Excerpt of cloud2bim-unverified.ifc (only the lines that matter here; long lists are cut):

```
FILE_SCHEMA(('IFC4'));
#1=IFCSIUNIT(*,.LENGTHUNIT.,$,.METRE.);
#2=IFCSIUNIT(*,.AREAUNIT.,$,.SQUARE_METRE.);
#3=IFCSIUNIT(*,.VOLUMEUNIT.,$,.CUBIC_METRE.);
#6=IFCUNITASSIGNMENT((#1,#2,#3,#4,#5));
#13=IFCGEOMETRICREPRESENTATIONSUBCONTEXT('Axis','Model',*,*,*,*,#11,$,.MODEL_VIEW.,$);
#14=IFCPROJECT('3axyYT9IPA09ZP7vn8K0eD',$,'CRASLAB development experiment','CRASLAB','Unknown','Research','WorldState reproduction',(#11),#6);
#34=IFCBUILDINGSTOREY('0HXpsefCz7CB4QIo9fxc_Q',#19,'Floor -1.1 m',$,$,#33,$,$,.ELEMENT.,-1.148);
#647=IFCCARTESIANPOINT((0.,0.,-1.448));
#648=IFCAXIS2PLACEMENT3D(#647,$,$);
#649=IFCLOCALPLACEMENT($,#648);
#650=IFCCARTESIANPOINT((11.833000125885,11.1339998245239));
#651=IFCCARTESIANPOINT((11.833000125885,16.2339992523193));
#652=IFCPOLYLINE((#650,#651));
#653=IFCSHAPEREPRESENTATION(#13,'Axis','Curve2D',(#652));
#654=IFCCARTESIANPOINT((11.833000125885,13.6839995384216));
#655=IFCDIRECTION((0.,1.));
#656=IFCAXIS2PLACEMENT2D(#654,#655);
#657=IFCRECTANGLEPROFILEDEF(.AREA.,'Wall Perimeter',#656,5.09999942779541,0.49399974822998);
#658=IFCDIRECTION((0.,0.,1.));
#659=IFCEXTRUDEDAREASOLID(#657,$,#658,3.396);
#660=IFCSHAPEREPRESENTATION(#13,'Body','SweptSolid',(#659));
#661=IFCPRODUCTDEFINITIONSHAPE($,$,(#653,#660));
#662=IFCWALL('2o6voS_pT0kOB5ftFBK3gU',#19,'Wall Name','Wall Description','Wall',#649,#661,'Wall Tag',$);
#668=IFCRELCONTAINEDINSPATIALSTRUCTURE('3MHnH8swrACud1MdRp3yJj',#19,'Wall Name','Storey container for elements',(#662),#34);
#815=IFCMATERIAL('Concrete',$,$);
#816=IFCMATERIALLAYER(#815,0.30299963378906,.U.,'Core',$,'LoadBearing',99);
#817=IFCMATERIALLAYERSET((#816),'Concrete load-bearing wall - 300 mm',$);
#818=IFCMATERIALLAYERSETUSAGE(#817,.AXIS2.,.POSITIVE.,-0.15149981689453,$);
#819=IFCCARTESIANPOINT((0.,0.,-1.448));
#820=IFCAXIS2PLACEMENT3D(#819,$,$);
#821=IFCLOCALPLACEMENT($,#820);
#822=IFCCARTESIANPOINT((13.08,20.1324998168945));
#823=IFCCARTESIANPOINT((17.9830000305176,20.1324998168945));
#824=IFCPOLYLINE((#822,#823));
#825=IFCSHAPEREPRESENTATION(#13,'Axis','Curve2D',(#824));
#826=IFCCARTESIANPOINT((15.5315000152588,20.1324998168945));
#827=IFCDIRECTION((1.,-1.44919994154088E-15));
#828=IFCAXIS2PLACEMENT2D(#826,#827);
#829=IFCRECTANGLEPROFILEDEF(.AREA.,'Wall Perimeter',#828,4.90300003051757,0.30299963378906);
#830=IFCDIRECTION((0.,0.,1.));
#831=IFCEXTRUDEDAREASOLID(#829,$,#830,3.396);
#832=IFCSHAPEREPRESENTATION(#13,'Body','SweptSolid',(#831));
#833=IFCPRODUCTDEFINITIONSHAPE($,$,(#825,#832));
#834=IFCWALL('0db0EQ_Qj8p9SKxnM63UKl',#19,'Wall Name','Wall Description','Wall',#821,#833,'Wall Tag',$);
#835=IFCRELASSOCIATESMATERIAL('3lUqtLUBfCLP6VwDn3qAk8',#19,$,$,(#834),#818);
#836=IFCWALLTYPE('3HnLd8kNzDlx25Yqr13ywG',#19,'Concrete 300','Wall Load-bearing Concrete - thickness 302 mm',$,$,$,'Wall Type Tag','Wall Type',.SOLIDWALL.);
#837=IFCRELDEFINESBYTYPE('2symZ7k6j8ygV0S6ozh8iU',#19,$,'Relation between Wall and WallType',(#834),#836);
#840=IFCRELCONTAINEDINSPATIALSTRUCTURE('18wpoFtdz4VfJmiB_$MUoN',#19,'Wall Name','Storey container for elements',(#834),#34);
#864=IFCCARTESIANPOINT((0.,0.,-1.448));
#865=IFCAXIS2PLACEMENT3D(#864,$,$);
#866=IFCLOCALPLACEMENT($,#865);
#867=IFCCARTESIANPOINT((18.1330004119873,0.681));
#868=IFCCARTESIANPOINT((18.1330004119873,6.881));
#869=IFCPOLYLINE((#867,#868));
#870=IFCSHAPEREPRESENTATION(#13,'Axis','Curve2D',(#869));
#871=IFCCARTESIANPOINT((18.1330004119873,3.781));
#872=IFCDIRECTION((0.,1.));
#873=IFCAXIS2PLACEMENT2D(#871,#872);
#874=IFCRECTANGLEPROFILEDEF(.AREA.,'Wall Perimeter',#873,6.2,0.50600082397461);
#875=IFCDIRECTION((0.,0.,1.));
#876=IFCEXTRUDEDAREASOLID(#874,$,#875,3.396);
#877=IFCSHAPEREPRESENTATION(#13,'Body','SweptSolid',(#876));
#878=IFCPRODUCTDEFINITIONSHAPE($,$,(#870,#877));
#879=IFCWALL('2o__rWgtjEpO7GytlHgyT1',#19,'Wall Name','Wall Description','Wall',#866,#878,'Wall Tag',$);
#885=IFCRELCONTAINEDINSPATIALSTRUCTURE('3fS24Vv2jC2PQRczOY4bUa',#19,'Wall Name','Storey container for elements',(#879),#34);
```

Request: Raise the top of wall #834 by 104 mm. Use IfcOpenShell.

```python
import ifcopenshell
import ifcopenshell.geom
import ifcopenshell.util.shape
import ifcopenshell.util.unit

model = ifcopenshell.open("cloud2bim-unverified.ifc")
unit_scale = ifcopenshell.util.unit.calculate_unit_scale(model)
settings = ifcopenshell.geom.settings()


def volume(element):
    """Net volume in cubic metres, openings subtracted."""
    shape = ifcopenshell.geom.create_shape(settings, element)
    return ifcopenshell.util.shape.get_volume(shape.geometry)


wall = model.by_guid("0db0EQ_Qj8p9SKxnM63UKl")
before = volume(wall)

body = next(r for r in wall.Representation.Representations if r.RepresentationIdentifier == "Body")
solid = body.Items[0]
old_height = solid.Depth
solid.Depth += 0.104 / unit_scale
after = volume(wall)

print(f"height {old_height:g} -> {solid.Depth:g}, volume {before:.3f} -> {after:.3f} m3")

model.write("cloud2bim-unverified_v2.ifc")
```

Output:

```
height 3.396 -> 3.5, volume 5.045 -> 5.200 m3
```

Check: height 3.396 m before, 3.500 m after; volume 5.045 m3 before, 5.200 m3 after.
